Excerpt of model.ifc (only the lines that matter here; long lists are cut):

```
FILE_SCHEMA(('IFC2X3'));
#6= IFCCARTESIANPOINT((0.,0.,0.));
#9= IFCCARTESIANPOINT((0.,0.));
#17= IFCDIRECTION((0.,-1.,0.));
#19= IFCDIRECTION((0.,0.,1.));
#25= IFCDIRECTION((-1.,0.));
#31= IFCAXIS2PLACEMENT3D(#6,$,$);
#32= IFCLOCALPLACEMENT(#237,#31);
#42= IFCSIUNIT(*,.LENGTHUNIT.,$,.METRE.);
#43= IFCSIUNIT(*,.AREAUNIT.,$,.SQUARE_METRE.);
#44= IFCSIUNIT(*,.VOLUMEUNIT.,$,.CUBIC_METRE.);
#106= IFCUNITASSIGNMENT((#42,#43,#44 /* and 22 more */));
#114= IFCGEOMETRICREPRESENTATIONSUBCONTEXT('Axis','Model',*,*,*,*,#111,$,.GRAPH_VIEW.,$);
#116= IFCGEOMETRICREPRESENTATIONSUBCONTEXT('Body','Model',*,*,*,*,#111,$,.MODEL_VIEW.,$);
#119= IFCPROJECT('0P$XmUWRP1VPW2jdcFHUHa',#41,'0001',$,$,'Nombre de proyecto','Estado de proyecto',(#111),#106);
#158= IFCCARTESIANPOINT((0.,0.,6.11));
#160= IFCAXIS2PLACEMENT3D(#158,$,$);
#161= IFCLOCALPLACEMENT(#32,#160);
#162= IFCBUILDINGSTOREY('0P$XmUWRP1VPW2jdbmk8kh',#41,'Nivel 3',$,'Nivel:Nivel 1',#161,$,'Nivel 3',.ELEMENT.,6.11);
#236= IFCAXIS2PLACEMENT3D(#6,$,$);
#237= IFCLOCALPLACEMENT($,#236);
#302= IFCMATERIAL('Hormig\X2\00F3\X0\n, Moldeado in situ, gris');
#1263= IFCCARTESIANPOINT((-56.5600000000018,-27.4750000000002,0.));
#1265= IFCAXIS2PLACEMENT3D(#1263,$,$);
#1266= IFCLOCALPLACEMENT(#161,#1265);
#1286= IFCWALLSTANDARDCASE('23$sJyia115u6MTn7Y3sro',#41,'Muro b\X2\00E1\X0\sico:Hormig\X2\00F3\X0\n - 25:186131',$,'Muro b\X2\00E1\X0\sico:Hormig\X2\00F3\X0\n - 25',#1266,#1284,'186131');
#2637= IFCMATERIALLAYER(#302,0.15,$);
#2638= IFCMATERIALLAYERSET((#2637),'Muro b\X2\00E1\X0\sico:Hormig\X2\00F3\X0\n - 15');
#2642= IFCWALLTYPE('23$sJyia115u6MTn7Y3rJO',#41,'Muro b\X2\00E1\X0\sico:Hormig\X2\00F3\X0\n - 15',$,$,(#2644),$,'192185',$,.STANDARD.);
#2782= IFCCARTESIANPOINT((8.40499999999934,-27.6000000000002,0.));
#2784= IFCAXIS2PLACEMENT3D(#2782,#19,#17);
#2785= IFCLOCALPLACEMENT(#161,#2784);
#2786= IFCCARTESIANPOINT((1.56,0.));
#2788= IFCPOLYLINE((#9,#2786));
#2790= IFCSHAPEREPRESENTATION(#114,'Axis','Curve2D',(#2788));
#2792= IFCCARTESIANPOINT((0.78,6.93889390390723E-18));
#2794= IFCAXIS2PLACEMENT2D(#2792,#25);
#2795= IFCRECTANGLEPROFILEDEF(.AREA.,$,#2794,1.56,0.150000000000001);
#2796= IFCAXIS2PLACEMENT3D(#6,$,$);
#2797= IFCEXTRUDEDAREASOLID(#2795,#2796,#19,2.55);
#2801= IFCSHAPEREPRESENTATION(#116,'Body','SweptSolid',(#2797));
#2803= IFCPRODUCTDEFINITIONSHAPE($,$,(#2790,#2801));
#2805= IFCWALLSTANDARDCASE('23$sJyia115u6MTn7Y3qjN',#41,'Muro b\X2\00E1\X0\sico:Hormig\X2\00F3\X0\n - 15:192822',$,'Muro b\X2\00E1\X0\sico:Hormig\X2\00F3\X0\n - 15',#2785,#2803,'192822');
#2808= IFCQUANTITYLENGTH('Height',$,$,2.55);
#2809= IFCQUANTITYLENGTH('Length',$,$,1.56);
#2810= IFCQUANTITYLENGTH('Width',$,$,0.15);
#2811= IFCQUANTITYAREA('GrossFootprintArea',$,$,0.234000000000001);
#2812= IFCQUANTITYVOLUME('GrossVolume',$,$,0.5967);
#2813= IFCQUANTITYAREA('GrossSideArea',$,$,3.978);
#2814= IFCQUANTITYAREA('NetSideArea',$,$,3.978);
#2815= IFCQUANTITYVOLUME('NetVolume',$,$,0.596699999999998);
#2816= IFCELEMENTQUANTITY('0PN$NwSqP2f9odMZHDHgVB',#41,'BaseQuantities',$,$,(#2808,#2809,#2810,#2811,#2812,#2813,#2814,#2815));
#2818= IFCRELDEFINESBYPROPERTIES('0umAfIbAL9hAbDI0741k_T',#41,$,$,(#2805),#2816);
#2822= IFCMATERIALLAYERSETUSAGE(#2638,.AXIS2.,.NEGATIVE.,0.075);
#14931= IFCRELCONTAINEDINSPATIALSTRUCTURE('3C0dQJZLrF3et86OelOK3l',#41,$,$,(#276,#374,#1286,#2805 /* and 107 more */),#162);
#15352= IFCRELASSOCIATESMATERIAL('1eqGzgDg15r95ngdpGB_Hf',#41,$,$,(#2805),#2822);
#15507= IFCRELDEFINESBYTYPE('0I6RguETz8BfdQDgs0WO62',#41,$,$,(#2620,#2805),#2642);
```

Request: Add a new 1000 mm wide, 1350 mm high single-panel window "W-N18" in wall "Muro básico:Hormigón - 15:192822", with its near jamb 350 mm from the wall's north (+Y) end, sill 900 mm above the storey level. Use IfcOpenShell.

```python
import numpy as np
import ifcopenshell
import ifcopenshell.api.feature
import ifcopenshell.api.geometry
import ifcopenshell.api.pset
import ifcopenshell.api.root
import ifcopenshell.api.spatial
import ifcopenshell.api.type
import ifcopenshell.geom
import ifcopenshell.util.element
import ifcopenshell.util.placement
import ifcopenshell.util.representation
import ifcopenshell.util.shape
import ifcopenshell.util.unit

model = ifcopenshell.open("model.ifc")
unit_scale = ifcopenshell.util.unit.calculate_unit_scale(model)
area_scale = ifcopenshell.util.unit.calculate_unit_scale(model, "AREAUNIT")
volume_scale = ifcopenshell.util.unit.calculate_unit_scale(model, "VOLUMEUNIT")
settings = ifcopenshell.geom.settings()


def volume(element):
    """Net volume in cubic metres, openings subtracted."""
    shape = ifcopenshell.geom.create_shape(settings, element)
    return ifcopenshell.util.shape.get_volume(shape.geometry)


wall = model.by_id(2805)
storey = ifcopenshell.util.element.get_container(wall, ifc_class="IfcBuildingStorey")
context = ifcopenshell.util.representation.get_context(model, "Model", "Body", "MODEL_VIEW")
before = volume(wall)

width, height, from_end, sill = 1, 1.35, 0.35, 0.9  # metres

# The wall runs along its own X axis, and the end named is its -X end.
wall_shape = ifcopenshell.geom.create_shape(settings, wall)
x, y, z = ifcopenshell.util.shape.get_vertices(wall_shape.geometry).T
start = x.min() + from_end
face, thickness = float(y.min()), float(y.max() - y.min())
wall_matrix = ifcopenshell.util.placement.get_local_placement(wall.ObjectPlacement)
level = ifcopenshell.util.placement.get_local_placement(storey.ObjectPlacement)[2, 3]


def in_wall(x, y):
    """Placement at x, y metres in the wall's axes, at sill height."""
    matrix = wall_matrix.copy()
    matrix[:, 3] = wall_matrix @ np.array([x / unit_scale, y / unit_scale, 0.0, 1.0])
    matrix[2, 3] = level + sill / unit_scale
    return matrix


# Opening: a box that overshoots both wall faces by 50 mm.
opening = ifcopenshell.api.root.create_entity(model, ifc_class="IfcOpeningElement")
box = ifcopenshell.api.geometry.add_wall_representation(
    model, context=context, length=width, height=height, thickness=thickness + 0.1
)
ifcopenshell.api.geometry.assign_representation(model, product=opening, representation=box)
ifcopenshell.api.geometry.edit_object_placement(model, product=opening, matrix=in_wall(start, face - 0.05), is_si=False)
ifcopenshell.api.feature.add_feature(model, feature=opening, element=wall)

window = ifcopenshell.api.root.create_entity(model, ifc_class="IfcWindow", name="W-N18")
window.OverallWidth, window.OverallHeight = width / unit_scale, height / unit_scale
body = ifcopenshell.api.geometry.add_window_representation(
    model,
    context=context,
    overall_width=window.OverallWidth,
    overall_height=window.OverallHeight,
    partition_type="SINGLE_PANEL",
)
ifcopenshell.api.geometry.assign_representation(model, product=window, representation=body)
ifcopenshell.api.spatial.assign_container(model, products=[window], relating_structure=storey)
fills = ifcopenshell.api.feature.add_filling(model, opening=opening, element=window)
fills.OwnerHistory = window.OwnerHistory  # required in IFC2X3

# IFC2X3 keeps the operation on the window style.
style = ifcopenshell.api.root.create_entity(model, ifc_class="IfcWindowStyle", name="W-N18")
style.OperationType, style.ConstructionType = "SINGLE_PANEL", "NOTDEFINED"
style.ParameterTakesPrecedence = style.Sizeable = False
ifcopenshell.api.type.assign_type(model, related_objects=[window], relating_type=style)

# Centre the window in the wall's thickness.
ifcopenshell.api.geometry.edit_object_placement(model, product=window, matrix=in_wall(start, face), is_si=False)
window_shape = ifcopenshell.geom.create_shape(settings, window)
depth = ifcopenshell.util.shape.get_vertices(window_shape.geometry)[:, 1]
offset = face + thickness / 2 - (depth.min() + depth.max()) / 2
ifcopenshell.api.geometry.edit_object_placement(model, product=window, matrix=in_wall(start, offset), is_si=False)

after = volume(wall)

# Update the wall's stored quantities.
qto = model.by_id(ifcopenshell.util.element.get_pset(wall, "BaseQuantities", should_inherit=False)["id"])
ifcopenshell.api.pset.edit_qto(model, qto=qto, properties={
    "NetSideArea": after / thickness / area_scale,
    "NetVolume": after / volume_scale,
})

print(f"wall volume {before:.3f} -> {after:.3f} m3")

model.write("model_rev.ifc")
```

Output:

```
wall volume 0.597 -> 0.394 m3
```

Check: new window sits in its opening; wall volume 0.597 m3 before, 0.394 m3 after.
